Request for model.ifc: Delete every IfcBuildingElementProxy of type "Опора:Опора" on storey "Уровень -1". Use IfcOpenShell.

First a look at what the model holds.

```python
import ifcopenshell
import ifcopenshell.util.element

model = ifcopenshell.open("model.ifc")
print(model.schema)
storey = next(s for s in model.by_type("IfcBuildingStorey") if s.Name == "Уровень -1")
proxies = [e for e in ifcopenshell.util.element.get_decomposition(storey) if e.is_a("IfcBuildingElementProxy")]
seen = {}
for e in proxies:
    element_type = ifcopenshell.util.element.get_type(e)
    name = element_type.Name if element_type not in (None, e) else None
    seen[name] = seen.get(name, 0) + 1
for name, count in sorted(seen.items(), key=str):
    print(count, "x", name)
```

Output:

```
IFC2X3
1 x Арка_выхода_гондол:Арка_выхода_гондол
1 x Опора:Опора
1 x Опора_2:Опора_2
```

```python
import ifcopenshell
import ifcopenshell.api.root
import ifcopenshell.util.element

model = ifcopenshell.open("model.ifc")

storey = next(s for s in model.by_type("IfcBuildingStorey") if s.Name == "Уровень -1")
proxies = [e for e in ifcopenshell.util.element.get_decomposition(storey) if e.is_a("IfcBuildingElementProxy")]
targets = [e for e in proxies if (t := ifcopenshell.util.element.get_type(e)) not in (None, e) and t.Name == "Опора:Опора"]

for e in targets:
    ifcopenshell.api.root.remove_product(model, product=e)
print(len(targets), "removed")

model.write("model_v2.ifc")
```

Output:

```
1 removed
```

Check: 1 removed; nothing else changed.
